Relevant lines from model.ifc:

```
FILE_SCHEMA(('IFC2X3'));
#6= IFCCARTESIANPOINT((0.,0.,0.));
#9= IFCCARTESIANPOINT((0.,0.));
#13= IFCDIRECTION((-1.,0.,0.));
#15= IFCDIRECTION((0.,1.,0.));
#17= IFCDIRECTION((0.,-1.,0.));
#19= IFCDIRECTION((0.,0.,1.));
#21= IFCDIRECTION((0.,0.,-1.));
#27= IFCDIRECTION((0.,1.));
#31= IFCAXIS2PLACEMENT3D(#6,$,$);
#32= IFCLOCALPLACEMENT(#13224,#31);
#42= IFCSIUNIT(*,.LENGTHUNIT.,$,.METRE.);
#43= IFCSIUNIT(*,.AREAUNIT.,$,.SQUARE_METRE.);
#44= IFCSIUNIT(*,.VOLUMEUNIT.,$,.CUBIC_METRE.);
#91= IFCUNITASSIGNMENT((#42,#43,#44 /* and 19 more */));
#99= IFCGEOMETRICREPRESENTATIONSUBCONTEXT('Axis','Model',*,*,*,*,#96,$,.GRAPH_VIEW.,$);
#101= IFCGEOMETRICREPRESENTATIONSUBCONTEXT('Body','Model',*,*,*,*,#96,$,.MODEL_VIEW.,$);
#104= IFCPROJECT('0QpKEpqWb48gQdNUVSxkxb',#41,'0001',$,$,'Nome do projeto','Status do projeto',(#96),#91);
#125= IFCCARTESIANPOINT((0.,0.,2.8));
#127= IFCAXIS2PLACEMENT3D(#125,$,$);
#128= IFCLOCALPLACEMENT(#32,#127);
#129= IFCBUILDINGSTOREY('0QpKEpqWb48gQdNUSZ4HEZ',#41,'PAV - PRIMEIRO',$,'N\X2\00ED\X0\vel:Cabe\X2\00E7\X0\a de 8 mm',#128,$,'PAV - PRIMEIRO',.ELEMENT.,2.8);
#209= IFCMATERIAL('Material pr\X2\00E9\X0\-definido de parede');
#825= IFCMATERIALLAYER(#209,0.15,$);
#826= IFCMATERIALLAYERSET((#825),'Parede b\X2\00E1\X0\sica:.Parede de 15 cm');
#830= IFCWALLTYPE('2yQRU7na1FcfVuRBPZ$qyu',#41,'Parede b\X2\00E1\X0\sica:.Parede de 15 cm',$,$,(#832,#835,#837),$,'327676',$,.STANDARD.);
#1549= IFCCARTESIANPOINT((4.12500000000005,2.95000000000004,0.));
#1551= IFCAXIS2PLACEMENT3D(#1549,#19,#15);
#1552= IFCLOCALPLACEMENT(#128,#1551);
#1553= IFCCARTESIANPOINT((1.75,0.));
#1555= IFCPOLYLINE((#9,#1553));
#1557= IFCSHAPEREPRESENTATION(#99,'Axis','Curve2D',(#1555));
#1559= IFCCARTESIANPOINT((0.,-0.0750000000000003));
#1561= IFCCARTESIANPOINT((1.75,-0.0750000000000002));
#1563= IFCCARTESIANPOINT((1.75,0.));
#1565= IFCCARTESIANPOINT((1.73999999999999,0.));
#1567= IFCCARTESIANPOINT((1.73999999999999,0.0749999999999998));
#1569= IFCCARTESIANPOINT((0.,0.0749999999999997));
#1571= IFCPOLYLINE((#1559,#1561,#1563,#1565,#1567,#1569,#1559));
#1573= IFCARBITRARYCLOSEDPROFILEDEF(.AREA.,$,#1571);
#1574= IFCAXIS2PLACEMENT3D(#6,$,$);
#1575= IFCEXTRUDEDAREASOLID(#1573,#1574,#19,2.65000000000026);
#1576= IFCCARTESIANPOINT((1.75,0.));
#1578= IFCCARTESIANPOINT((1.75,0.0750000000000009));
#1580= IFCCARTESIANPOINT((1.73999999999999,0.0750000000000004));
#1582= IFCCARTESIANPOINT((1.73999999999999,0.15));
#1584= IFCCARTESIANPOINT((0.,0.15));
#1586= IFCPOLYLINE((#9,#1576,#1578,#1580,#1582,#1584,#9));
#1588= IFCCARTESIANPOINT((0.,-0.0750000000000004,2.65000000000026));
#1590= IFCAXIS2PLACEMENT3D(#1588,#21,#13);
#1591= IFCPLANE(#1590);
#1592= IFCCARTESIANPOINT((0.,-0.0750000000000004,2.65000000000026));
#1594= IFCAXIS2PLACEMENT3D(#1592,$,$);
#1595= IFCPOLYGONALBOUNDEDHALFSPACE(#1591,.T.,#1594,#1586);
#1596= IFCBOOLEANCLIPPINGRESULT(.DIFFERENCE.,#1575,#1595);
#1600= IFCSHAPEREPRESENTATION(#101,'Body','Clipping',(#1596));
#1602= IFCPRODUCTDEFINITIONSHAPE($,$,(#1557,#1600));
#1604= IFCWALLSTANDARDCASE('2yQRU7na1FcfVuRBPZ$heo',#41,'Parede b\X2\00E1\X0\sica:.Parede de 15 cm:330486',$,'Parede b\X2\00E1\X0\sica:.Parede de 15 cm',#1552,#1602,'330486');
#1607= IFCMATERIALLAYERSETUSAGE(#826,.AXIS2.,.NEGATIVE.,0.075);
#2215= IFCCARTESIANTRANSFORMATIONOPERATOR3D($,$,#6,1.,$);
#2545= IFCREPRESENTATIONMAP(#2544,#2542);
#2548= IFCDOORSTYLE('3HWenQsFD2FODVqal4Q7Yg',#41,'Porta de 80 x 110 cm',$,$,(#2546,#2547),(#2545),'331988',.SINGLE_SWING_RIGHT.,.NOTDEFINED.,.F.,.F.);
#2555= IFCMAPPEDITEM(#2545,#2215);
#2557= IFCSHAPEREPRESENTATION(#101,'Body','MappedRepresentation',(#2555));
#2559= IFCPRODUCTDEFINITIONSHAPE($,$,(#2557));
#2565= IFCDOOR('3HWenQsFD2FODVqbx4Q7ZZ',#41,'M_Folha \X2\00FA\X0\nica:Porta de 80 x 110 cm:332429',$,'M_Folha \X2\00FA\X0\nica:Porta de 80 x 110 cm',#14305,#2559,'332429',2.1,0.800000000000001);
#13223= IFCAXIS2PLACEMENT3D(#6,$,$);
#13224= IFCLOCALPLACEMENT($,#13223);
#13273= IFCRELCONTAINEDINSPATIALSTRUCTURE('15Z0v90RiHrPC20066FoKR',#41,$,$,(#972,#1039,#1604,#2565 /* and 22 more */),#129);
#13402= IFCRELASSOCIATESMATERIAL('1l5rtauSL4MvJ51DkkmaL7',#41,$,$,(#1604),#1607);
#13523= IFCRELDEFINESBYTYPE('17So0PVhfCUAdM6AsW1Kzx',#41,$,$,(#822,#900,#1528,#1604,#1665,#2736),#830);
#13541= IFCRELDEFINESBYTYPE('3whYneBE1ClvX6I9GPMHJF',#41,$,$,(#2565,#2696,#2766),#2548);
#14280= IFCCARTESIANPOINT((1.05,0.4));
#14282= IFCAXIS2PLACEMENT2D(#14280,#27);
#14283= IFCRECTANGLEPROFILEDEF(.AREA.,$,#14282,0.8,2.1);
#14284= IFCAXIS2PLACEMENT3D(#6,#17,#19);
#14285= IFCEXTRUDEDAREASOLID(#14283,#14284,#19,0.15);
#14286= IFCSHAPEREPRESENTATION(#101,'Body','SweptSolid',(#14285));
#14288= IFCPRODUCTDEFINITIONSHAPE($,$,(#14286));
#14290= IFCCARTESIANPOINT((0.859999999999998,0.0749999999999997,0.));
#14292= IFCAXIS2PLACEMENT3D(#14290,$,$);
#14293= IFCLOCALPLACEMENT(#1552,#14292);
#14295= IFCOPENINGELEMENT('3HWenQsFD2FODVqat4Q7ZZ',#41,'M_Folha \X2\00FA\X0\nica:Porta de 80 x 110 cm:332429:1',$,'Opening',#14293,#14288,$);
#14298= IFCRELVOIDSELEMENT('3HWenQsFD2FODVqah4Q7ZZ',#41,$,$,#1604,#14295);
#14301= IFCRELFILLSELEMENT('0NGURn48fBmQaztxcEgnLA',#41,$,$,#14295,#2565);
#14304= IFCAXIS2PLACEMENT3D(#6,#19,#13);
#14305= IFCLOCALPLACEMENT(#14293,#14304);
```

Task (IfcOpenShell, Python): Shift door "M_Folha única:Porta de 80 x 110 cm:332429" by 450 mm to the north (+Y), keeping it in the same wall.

```python
import ifcopenshell
import ifcopenshell.api.geometry
import ifcopenshell.util.placement

model = ifcopenshell.open("model.ifc")

door = model.by_guid("3HWenQsFD2FODVqbx4Q7ZZ")
opening = door.FillsVoids[0].RelatingOpeningElement
wall = opening.VoidsElements[0].RelatingBuildingElement

wall_matrix = ifcopenshell.util.placement.get_local_placement(wall.ObjectPlacement)
shift = wall_matrix[:3, 0] * 0.45
before = ifcopenshell.util.placement.get_local_placement(door.ObjectPlacement)[:3, 3].copy()

# The door is placed relative to its opening, so it follows when the opening moves.
matrix = ifcopenshell.util.placement.get_local_placement(opening.ObjectPlacement)
matrix[:3, 3] += shift
ifcopenshell.api.geometry.edit_object_placement(
    model, product=opening, matrix=matrix, is_si=False, should_transform_children=True
)

after = ifcopenshell.util.placement.get_local_placement(door.ObjectPlacement)[:3, 3]
print("door moved by", (after - before).round(3) + 0.0)

model.write("model_v2.ifc")
```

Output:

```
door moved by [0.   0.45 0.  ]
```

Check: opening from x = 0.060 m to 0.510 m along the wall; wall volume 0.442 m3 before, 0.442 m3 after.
